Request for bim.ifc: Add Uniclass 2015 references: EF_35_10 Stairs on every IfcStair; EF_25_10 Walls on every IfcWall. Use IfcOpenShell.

First a look at what the model holds.

```python
import ifcopenshell

model = ifcopenshell.open("bim.ifc")
print(model.schema)
print("classifications:", [c.Name for c in model.by_type("IfcClassification")])
for ifc_class in ("IfcDoor", "IfcRoof", "IfcStair", "IfcWall", "IfcWindow"):
    print(ifc_class, len(model.by_type(ifc_class)))
```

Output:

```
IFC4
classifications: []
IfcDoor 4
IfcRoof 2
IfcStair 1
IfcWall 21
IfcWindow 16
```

```python
import ifcopenshell
import ifcopenshell.api.classification

model = ifcopenshell.open("bim.ifc")

system = ifcopenshell.api.classification.add_classification(model, classification="Uniclass 2015")

codes = {
    "IfcStair": ("EF_35_10", "Stairs"),
    "IfcWall": ("EF_25_10", "Walls"),
}
for ifc_class, (code, name) in codes.items():
    products = model.by_type(ifc_class)
    ifcopenshell.api.classification.add_reference(
        model, products=products, classification=system, identification=code, name=name
    )
    print(code, len(products))

model.write("bim_updated.ifc")
```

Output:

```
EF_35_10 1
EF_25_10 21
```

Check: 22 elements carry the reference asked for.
